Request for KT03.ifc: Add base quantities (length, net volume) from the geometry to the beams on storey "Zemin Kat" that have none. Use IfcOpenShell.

First a look at what the model holds.

```python
import ifcopenshell
import ifcopenshell.util.element
import ifcopenshell.util.unit

model = ifcopenshell.open("KT03.ifc")
print(model.schema)
for unit_type in ("LENGTHUNIT", "AREAUNIT", "VOLUMEUNIT"):
    print(unit_type, ifcopenshell.util.unit.calculate_unit_scale(model, unit_type))
storey = next(s for s in model.by_type("IfcBuildingStorey") if s.Name == "Zemin Kat")
beams = [e for e in ifcopenshell.util.element.get_decomposition(storey) if e.is_a("IfcBeam")]
for e in sorted(beams, key=lambda e: e.id()):
    print(e.id(), e.is_a(), e.Name, list(ifcopenshell.util.element.get_psets(e, qtos_only=True)), sep=" | ")
```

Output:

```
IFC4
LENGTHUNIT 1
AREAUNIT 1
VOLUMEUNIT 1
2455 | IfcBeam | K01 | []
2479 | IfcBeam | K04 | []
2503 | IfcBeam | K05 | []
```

```python
import ifcopenshell
import ifcopenshell.api.pset
import ifcopenshell.geom
import ifcopenshell.util.element
import ifcopenshell.util.shape
import ifcopenshell.util.unit

model = ifcopenshell.open("KT03.ifc")
unit_scale = ifcopenshell.util.unit.calculate_unit_scale(model)
volume_scale = ifcopenshell.util.unit.calculate_unit_scale(model, "VOLUMEUNIT")
settings = ifcopenshell.geom.settings()

storey = next(s for s in model.by_type("IfcBuildingStorey") if s.Name == "Zemin Kat")
beams = [e for e in ifcopenshell.util.element.get_decomposition(storey) if e.is_a("IfcBeam")]

for e in sorted(beams, key=lambda e: e.id()):
    if ifcopenshell.util.element.get_psets(e, qtos_only=True, should_inherit=False):
        continue
    # Geometry comes back in metres, in the element's own axes.
    shape = ifcopenshell.geom.create_shape(settings, e)
    values = {
        "Length": ifcopenshell.util.shape.get_max_xyz(shape.geometry) / unit_scale,
        "NetVolume": ifcopenshell.util.shape.get_volume(shape.geometry) / volume_scale,
    }
    qto = ifcopenshell.api.pset.add_qto(model, product=e, name="Qto_BeamBaseQuantities")
    ifcopenshell.api.pset.edit_qto(model, qto=qto, properties=values)
    print(e.id(), {k: round(v, 3) for k, v in values.items()})

model.write("KT03_edited.ifc")
```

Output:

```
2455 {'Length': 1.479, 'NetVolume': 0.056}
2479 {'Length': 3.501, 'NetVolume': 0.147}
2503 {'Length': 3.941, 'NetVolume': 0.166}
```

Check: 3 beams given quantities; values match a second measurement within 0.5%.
